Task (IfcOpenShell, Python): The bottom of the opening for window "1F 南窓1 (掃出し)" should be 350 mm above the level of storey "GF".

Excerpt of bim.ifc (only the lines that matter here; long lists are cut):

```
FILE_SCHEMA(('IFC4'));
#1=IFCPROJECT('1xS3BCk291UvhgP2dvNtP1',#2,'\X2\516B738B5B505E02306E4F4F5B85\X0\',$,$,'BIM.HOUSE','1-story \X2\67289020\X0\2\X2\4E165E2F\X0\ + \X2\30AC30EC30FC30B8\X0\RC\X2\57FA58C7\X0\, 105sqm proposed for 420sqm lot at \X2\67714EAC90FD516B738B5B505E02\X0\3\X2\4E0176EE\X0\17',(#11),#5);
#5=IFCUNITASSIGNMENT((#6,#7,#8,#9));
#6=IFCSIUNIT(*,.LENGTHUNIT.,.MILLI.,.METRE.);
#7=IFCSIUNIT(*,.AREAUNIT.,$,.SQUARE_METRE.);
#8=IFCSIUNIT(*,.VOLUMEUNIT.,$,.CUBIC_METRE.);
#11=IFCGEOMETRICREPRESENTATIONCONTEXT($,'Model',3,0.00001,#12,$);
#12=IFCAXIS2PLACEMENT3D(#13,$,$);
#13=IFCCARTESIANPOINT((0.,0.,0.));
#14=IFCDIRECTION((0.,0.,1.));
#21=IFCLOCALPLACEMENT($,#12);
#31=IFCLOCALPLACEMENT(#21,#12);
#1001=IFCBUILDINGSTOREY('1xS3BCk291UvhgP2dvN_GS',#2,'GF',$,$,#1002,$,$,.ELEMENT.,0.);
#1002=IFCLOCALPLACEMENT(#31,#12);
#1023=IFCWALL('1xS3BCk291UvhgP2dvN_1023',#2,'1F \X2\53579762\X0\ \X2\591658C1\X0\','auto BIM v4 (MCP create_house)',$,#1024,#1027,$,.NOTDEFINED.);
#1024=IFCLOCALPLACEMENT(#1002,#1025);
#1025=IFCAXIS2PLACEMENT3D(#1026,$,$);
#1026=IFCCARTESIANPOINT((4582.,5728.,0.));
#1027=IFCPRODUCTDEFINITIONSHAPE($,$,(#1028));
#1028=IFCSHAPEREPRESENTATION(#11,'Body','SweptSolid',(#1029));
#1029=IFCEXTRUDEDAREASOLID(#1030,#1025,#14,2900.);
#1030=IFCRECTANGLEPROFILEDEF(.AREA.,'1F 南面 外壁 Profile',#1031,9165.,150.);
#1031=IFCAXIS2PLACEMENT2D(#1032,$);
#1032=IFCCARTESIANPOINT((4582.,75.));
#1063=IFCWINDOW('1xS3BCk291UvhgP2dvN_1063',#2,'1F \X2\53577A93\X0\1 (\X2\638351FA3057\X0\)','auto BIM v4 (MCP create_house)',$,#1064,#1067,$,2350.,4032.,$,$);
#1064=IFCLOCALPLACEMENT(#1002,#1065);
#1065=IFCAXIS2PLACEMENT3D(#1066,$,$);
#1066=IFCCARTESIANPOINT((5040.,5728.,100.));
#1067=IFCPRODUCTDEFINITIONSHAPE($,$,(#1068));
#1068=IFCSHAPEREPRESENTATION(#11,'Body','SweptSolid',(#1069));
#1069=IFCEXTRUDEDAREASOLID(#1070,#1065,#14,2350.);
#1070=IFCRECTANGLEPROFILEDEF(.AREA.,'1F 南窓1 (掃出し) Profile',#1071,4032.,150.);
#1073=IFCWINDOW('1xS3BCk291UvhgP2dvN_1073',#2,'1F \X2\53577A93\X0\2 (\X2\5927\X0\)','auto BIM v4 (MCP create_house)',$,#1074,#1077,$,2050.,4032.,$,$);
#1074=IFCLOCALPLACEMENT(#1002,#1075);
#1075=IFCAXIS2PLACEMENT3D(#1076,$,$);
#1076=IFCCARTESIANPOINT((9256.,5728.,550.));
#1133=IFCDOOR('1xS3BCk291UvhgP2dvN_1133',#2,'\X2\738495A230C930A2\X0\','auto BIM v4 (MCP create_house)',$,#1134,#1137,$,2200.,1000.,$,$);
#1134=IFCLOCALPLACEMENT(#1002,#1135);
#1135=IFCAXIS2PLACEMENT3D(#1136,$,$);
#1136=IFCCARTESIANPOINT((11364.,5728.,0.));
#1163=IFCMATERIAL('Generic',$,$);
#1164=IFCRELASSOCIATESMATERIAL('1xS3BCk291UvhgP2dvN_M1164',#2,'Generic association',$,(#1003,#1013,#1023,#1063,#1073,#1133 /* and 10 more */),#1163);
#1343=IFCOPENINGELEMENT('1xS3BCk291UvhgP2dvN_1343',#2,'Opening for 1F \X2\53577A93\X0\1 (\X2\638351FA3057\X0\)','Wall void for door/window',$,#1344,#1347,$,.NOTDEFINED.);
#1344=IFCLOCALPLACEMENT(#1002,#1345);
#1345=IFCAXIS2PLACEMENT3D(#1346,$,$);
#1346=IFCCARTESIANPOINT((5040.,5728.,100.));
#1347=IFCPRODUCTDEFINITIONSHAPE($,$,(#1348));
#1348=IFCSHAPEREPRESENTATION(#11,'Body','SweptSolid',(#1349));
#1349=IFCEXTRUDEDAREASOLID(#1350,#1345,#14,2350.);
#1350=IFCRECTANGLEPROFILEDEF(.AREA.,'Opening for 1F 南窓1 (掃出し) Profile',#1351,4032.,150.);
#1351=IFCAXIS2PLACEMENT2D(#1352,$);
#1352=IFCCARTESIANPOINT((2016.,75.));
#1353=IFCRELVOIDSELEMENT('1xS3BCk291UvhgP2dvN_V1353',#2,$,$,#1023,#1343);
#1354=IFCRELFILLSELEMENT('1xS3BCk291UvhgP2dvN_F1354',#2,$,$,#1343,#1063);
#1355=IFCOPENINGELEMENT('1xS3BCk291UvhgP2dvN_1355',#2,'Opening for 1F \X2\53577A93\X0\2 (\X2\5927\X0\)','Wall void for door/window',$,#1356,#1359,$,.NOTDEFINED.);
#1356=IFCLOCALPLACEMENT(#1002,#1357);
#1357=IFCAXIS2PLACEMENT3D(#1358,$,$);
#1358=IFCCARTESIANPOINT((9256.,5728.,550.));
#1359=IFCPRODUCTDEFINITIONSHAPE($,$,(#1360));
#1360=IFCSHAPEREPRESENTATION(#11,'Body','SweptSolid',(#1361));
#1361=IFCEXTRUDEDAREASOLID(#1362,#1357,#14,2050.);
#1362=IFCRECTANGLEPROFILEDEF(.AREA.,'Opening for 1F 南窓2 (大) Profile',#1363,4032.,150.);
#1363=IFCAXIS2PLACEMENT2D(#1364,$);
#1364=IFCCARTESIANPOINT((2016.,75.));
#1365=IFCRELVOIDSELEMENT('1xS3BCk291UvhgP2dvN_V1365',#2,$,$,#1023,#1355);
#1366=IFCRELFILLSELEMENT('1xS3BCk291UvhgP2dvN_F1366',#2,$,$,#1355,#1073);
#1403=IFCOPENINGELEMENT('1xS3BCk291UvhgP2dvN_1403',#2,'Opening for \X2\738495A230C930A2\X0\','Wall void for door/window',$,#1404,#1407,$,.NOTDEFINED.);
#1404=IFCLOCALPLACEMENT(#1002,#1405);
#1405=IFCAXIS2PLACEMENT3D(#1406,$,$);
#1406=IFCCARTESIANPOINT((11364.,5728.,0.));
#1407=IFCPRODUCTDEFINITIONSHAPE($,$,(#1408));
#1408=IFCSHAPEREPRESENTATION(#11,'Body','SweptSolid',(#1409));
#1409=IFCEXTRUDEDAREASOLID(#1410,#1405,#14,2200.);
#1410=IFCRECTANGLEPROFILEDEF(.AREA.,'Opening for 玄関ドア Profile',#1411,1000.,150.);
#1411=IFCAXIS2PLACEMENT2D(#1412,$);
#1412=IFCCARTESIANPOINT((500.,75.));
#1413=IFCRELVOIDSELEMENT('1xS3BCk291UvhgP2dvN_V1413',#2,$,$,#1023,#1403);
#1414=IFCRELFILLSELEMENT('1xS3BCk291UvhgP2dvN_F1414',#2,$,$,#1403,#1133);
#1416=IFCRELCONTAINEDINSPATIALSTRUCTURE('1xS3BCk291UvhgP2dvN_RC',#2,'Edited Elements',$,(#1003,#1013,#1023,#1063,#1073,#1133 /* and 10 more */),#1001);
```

```python
import numpy as np
import ifcopenshell
import ifcopenshell.api.geometry
import ifcopenshell.geom
import ifcopenshell.util.element
import ifcopenshell.util.placement
import ifcopenshell.util.shape
import ifcopenshell.util.unit

model = ifcopenshell.open("bim.ifc")
unit_scale = ifcopenshell.util.unit.calculate_unit_scale(model)

window = model.by_guid("1xS3BCk291UvhgP2dvN_1063")
opening = window.FillsVoids[0].RelatingOpeningElement
storey = ifcopenshell.util.element.get_container(window, ifc_class="IfcBuildingStorey")
level = ifcopenshell.util.placement.get_local_placement(storey.ObjectPlacement)[2, 3]

# The opening's origin need not be at the sill, so measure its lowest point.
shape = ifcopenshell.geom.create_shape(ifcopenshell.geom.settings(), opening)
bottom = ifcopenshell.util.shape.get_shape_bottom_elevation(shape, shape.geometry) / unit_scale
dz = level + 350.0 - bottom

shift = np.array([0.0, 0.0, dz])
# The window is not placed relative to its opening, so move both.
for product in (opening, window):
    matrix = ifcopenshell.util.placement.get_local_placement(product.ObjectPlacement)
    matrix[:3, 3] += shift
    ifcopenshell.api.geometry.edit_object_placement(model, product=product, matrix=matrix, is_si=False)

print(f"moved by {dz * unit_scale:+.3f} m")

model.write("bim_updated.ifc")
```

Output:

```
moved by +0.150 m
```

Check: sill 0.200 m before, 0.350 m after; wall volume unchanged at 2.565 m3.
